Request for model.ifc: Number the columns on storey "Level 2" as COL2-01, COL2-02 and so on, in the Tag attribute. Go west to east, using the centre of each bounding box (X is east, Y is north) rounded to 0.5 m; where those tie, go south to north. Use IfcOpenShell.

First a look at what the model holds.

```python
import ifcopenshell
import ifcopenshell.util.element
import ifcopenshell.util.placement

model = ifcopenshell.open("model.ifc")
print(model.schema)
storey = next(s for s in model.by_type("IfcBuildingStorey") if s.Name == "Level 2")
columns = [e for e in ifcopenshell.util.element.get_decomposition(storey) if e.is_a("IfcColumn")]
for e in sorted(columns, key=lambda e: e.id()):
    origin = ifcopenshell.util.placement.get_local_placement(e.ObjectPlacement)[:3, 3]
    print(e.id(), e.Tag, e.Name, origin.round(2) + 0.0, sep=" | ")
```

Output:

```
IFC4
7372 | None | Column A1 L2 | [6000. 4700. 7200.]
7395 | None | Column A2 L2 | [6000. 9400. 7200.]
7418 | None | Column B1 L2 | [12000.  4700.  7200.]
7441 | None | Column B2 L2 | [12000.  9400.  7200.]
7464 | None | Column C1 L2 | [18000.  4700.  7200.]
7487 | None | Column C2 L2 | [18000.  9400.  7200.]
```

```python
import ifcopenshell
import ifcopenshell.geom
import ifcopenshell.util.element
import ifcopenshell.util.shape

model = ifcopenshell.open("model.ifc")
settings = ifcopenshell.geom.settings()
settings.set("use-world-coords", True)


def centre(element):
    shape = ifcopenshell.geom.create_shape(settings, element)
    return ifcopenshell.util.shape.get_bbox_centroid(shape.geometry)


storey = next(s for s in model.by_type("IfcBuildingStorey") if s.Name == "Level 2")
columns = [e for e in ifcopenshell.util.element.get_decomposition(storey) if e.is_a("IfcColumn")]

# Insertion points can sit at a corner or the storey origin, so sort by the geometry (in metres).
centres = {e: centre(e) for e in columns}
columns.sort(key=lambda e: (round(centres[e][0] / 0.5), centres[e][1]))

for i, e in enumerate(columns, start=1):
    number = f"COL2-{i:02d}"
    e.Tag = number
    print(e.id(), number)

model.write("model-out.ifc")
```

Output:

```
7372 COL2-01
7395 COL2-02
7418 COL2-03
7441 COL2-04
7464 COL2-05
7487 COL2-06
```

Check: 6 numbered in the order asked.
